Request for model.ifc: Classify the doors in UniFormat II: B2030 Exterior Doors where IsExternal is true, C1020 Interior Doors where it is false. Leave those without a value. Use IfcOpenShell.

First a look at what the model holds.

```python
import ifcopenshell
import ifcopenshell.util.element

model = ifcopenshell.open("model.ifc")
print(model.schema)
print("classifications:", [c.Name for c in model.by_type("IfcClassification")])
values = [ifcopenshell.util.element.get_pset(e, "Pset_DoorCommon", "IsExternal") for e in model.by_type("IfcDoor")]
for value in (True, False, None):
    print("IsExternal", value, values.count(value))
```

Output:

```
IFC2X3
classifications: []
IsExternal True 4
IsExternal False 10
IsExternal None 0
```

```python
import ifcopenshell
import ifcopenshell.api.classification
import ifcopenshell.util.element

model = ifcopenshell.open("model.ifc")

# IFC2X3 requires Source and Edition and has no link from the project to the system.
system = model.create_entity("IfcClassification", Source="ASTM", Edition="E1557", Name="UniFormat II")

doors = model.by_type("IfcDoor")
external = {e: ifcopenshell.util.element.get_pset(e, "Pset_DoorCommon", "IsExternal") for e in doors}
for flag, code, name in ((True, "B2030", "Exterior Doors"), (False, "C1020", "Interior Doors")):
    products = [e for e in doors if external[e] is flag]
    ifcopenshell.api.classification.add_reference(
        model, products=products, classification=system, identification=code, name=name
    )
    print(code, len(products))

model.write("model_rev.ifc")
```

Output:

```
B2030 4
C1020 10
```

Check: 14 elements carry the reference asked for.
